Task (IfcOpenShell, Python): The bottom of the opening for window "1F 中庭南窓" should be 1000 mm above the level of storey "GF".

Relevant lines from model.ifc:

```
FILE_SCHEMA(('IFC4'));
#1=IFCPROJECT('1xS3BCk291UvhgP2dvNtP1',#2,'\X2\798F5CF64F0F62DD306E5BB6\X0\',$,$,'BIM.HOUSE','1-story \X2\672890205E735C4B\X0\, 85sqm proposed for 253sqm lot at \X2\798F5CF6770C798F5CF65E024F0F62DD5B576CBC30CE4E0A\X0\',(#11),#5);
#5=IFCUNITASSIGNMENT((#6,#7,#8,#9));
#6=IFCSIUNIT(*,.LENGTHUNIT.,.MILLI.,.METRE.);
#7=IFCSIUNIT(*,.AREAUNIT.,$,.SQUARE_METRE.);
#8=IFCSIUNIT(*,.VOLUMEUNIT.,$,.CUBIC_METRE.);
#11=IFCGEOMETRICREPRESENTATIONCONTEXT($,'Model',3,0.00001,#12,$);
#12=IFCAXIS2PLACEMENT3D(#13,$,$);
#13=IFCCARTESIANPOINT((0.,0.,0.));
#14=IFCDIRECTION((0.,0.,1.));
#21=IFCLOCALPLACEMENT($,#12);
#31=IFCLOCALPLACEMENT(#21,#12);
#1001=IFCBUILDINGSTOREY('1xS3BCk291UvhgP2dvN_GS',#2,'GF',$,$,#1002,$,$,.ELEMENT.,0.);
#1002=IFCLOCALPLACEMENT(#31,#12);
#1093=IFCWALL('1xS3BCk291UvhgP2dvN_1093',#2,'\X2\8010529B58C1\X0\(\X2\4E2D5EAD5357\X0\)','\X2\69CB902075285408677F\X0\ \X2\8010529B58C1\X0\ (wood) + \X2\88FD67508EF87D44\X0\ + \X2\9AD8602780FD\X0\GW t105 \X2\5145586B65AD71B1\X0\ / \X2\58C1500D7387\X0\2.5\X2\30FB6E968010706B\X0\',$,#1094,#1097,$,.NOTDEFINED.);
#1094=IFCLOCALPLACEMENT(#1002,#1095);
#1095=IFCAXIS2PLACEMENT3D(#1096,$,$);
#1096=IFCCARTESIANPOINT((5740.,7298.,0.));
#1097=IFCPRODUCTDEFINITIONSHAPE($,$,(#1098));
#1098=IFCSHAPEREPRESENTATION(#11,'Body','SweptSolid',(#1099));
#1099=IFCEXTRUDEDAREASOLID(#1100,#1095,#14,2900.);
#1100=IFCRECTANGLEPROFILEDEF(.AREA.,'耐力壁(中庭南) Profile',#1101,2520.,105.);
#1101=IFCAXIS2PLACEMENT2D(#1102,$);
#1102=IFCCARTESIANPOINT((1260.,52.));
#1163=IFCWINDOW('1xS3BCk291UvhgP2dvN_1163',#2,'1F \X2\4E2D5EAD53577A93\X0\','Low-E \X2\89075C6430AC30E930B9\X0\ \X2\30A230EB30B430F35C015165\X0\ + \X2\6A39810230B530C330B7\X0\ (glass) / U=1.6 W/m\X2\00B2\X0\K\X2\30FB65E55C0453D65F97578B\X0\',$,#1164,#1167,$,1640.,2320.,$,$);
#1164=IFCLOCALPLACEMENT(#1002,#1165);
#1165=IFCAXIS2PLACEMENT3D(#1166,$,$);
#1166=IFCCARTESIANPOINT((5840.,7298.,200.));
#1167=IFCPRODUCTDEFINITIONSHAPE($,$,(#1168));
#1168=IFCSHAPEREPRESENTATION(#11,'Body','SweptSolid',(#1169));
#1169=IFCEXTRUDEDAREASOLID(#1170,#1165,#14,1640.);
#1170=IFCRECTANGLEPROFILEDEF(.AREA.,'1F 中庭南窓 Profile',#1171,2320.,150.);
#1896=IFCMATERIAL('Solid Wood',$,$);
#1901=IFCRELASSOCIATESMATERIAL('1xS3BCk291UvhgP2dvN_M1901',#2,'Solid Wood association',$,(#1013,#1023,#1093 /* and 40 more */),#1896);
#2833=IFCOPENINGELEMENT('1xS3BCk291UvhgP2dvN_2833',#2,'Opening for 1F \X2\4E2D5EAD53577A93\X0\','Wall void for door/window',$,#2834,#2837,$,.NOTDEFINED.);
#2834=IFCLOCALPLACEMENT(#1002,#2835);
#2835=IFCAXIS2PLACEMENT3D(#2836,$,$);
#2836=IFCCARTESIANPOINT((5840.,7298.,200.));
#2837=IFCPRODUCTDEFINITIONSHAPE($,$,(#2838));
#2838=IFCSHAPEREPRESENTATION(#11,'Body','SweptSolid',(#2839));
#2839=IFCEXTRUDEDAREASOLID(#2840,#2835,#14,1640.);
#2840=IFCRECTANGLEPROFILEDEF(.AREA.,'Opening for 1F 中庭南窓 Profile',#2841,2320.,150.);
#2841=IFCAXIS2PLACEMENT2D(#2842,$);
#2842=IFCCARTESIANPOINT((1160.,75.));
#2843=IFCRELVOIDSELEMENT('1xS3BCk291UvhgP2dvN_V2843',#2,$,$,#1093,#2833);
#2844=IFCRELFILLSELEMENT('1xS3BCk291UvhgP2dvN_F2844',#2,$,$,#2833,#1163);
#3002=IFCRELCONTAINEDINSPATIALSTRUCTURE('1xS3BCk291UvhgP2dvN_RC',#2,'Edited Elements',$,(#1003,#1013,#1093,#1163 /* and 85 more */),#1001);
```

```python
import numpy as np
import ifcopenshell
import ifcopenshell.api.geometry
import ifcopenshell.geom
import ifcopenshell.util.element
import ifcopenshell.util.placement
import ifcopenshell.util.shape
import ifcopenshell.util.unit

model = ifcopenshell.open("model.ifc")
unit_scale = ifcopenshell.util.unit.calculate_unit_scale(model)

window = model.by_id(1163)
opening = window.FillsVoids[0].RelatingOpeningElement
storey = ifcopenshell.util.element.get_container(window, ifc_class="IfcBuildingStorey")
level = ifcopenshell.util.placement.get_local_placement(storey.ObjectPlacement)[2, 3]

# The opening's origin need not be at the sill, so measure its lowest point.
shape = ifcopenshell.geom.create_shape(ifcopenshell.geom.settings(), opening)
bottom = ifcopenshell.util.shape.get_shape_bottom_elevation(shape, shape.geometry) / unit_scale
dz = level + 1 / unit_scale - bottom

shift = np.array([0.0, 0.0, dz])
# The window is not placed relative to its opening, so move both.
for product in (opening, window):
    matrix = ifcopenshell.util.placement.get_local_placement(product.ObjectPlacement)
    matrix[:3, 3] += shift
    ifcopenshell.api.geometry.edit_object_placement(model, product=product, matrix=matrix, is_si=False)

print(f"moved by {dz * unit_scale:+.3f} m")

model.write("model-out.ifc")
```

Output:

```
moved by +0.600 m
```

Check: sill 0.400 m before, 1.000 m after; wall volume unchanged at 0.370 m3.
